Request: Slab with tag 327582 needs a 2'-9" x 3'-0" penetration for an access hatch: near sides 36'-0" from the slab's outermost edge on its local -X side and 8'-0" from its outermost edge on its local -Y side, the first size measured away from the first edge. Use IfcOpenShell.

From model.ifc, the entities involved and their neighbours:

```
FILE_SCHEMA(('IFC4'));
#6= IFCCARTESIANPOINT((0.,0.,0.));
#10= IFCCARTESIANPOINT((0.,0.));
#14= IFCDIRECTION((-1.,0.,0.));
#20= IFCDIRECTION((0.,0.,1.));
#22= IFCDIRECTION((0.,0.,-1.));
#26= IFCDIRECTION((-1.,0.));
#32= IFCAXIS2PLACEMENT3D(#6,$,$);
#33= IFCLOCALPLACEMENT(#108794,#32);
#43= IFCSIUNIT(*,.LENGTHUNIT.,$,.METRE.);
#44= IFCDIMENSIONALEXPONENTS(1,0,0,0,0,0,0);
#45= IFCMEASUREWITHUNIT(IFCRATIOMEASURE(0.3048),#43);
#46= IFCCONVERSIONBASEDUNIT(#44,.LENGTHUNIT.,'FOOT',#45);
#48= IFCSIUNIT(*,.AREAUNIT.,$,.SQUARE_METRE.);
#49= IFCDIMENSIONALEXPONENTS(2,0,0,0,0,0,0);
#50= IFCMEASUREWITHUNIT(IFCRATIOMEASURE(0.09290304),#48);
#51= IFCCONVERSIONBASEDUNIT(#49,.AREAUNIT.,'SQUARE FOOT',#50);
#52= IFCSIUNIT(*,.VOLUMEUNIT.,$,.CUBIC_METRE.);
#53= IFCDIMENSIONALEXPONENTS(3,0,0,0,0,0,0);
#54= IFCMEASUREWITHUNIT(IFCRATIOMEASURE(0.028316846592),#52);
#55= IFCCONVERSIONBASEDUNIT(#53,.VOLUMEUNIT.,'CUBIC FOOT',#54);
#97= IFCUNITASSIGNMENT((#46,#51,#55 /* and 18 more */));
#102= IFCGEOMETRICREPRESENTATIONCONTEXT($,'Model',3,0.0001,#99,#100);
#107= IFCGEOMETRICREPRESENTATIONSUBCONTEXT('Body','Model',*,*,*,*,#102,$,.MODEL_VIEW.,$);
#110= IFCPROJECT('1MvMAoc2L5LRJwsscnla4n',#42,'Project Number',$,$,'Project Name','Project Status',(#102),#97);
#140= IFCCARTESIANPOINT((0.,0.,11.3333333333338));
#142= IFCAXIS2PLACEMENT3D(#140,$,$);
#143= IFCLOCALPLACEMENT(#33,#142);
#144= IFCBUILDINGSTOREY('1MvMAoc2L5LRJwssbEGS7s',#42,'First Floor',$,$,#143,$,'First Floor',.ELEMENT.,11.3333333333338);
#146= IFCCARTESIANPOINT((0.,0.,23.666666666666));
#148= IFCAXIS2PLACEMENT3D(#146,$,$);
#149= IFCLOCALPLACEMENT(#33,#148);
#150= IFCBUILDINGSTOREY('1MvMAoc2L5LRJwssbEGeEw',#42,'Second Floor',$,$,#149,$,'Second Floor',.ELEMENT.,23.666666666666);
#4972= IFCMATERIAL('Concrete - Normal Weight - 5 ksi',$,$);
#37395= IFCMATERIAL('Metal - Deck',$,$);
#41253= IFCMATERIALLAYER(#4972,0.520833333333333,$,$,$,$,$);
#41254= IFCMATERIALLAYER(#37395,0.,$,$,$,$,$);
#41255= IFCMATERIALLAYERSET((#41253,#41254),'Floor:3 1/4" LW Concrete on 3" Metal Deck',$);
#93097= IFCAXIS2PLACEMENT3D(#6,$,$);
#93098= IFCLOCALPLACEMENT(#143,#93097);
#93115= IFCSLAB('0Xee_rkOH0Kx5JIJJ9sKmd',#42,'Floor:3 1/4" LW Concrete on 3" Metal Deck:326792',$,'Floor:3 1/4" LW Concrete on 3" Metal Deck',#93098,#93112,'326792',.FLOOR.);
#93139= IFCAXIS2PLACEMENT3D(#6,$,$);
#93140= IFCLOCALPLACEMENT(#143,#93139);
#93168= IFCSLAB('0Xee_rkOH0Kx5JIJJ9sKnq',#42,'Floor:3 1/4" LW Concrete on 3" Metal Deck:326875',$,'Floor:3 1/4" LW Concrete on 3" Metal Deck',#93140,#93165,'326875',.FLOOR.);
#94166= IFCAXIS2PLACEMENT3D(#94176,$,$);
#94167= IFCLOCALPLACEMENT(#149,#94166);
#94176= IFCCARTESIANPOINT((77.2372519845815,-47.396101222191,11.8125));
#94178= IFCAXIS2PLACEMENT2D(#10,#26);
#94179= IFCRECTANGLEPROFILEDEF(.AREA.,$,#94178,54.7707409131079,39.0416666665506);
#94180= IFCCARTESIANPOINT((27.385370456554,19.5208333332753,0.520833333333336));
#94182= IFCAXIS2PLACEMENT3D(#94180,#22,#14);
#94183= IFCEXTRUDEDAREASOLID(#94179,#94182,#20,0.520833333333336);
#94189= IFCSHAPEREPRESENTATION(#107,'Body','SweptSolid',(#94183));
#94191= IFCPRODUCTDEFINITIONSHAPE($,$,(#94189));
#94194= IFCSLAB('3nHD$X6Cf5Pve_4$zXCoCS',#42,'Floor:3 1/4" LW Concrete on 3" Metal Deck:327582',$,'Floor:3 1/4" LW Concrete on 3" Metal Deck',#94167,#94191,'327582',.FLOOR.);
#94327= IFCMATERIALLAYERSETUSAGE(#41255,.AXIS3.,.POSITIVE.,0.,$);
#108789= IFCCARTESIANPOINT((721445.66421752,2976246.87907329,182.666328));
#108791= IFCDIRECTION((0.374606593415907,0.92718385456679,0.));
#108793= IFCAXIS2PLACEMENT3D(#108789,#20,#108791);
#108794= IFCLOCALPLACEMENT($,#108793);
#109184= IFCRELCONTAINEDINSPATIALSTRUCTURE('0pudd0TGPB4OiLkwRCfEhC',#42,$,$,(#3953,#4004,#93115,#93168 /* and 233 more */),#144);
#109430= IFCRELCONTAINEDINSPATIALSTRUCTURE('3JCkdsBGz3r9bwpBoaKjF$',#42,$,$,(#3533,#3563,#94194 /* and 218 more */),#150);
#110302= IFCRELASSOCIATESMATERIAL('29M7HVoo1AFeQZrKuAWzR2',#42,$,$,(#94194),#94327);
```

```python
import numpy as np
import ifcopenshell
import ifcopenshell.api.feature
import ifcopenshell.api.geometry
import ifcopenshell.api.root
import ifcopenshell.geom
import ifcopenshell.util.placement
import ifcopenshell.util.representation
import ifcopenshell.util.shape
import ifcopenshell.util.unit

model = ifcopenshell.open("model.ifc")
unit_scale = ifcopenshell.util.unit.calculate_unit_scale(model)
settings = ifcopenshell.geom.settings()


def volume(element):
    """Net volume in cubic metres, openings subtracted."""
    shape = ifcopenshell.geom.create_shape(settings, element)
    return ifcopenshell.util.shape.get_volume(shape.geometry)


slab = model.by_id(94194)
before = volume(slab)

# Extent in the slab's own axes, in metres. The edges named are its -X and -Y sides.
slab_shape = ifcopenshell.geom.create_shape(settings, slab)
vertices = ifcopenshell.util.shape.get_vertices(slab_shape.geometry)
x_min, y_min, bottom = vertices.min(axis=0)
top = vertices[:, 2].max()

opening = ifcopenshell.api.root.create_entity(model, ifc_class="IfcOpeningElement", name="Access hatch opening", predefined_type="OPENING")
context = ifcopenshell.util.representation.get_context(model, "Model", "Body", "MODEL_VIEW")
width, depth = 0.8382, 0.9144
outline = [(0.0, 0.0), (width, 0.0), (width, depth), (0.0, depth), (0.0, 0.0)]
# Overshoot both faces by 50 mm so the cut is clean.
shape = ifcopenshell.api.geometry.add_slab_representation(
    model, context=context, depth=top - bottom + 0.1, polyline=outline
)
ifcopenshell.api.geometry.assign_representation(model, product=opening, representation=shape)

matrix = ifcopenshell.util.placement.get_local_placement(slab.ObjectPlacement)
matrix[:, 3] = matrix @ np.append(np.array([x_min + 10.9728, y_min + 2.4384, bottom - 0.05]) / unit_scale, 1.0)
ifcopenshell.api.geometry.edit_object_placement(model, product=opening, matrix=matrix, is_si=False)
ifcopenshell.api.feature.add_feature(model, feature=opening, element=slab)

after = volume(slab)

print(f"slab volume {before:.3f} -> {after:.3f} m3")

model.write("model-out.ifc")
```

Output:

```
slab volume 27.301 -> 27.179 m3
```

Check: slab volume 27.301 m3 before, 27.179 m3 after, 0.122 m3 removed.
